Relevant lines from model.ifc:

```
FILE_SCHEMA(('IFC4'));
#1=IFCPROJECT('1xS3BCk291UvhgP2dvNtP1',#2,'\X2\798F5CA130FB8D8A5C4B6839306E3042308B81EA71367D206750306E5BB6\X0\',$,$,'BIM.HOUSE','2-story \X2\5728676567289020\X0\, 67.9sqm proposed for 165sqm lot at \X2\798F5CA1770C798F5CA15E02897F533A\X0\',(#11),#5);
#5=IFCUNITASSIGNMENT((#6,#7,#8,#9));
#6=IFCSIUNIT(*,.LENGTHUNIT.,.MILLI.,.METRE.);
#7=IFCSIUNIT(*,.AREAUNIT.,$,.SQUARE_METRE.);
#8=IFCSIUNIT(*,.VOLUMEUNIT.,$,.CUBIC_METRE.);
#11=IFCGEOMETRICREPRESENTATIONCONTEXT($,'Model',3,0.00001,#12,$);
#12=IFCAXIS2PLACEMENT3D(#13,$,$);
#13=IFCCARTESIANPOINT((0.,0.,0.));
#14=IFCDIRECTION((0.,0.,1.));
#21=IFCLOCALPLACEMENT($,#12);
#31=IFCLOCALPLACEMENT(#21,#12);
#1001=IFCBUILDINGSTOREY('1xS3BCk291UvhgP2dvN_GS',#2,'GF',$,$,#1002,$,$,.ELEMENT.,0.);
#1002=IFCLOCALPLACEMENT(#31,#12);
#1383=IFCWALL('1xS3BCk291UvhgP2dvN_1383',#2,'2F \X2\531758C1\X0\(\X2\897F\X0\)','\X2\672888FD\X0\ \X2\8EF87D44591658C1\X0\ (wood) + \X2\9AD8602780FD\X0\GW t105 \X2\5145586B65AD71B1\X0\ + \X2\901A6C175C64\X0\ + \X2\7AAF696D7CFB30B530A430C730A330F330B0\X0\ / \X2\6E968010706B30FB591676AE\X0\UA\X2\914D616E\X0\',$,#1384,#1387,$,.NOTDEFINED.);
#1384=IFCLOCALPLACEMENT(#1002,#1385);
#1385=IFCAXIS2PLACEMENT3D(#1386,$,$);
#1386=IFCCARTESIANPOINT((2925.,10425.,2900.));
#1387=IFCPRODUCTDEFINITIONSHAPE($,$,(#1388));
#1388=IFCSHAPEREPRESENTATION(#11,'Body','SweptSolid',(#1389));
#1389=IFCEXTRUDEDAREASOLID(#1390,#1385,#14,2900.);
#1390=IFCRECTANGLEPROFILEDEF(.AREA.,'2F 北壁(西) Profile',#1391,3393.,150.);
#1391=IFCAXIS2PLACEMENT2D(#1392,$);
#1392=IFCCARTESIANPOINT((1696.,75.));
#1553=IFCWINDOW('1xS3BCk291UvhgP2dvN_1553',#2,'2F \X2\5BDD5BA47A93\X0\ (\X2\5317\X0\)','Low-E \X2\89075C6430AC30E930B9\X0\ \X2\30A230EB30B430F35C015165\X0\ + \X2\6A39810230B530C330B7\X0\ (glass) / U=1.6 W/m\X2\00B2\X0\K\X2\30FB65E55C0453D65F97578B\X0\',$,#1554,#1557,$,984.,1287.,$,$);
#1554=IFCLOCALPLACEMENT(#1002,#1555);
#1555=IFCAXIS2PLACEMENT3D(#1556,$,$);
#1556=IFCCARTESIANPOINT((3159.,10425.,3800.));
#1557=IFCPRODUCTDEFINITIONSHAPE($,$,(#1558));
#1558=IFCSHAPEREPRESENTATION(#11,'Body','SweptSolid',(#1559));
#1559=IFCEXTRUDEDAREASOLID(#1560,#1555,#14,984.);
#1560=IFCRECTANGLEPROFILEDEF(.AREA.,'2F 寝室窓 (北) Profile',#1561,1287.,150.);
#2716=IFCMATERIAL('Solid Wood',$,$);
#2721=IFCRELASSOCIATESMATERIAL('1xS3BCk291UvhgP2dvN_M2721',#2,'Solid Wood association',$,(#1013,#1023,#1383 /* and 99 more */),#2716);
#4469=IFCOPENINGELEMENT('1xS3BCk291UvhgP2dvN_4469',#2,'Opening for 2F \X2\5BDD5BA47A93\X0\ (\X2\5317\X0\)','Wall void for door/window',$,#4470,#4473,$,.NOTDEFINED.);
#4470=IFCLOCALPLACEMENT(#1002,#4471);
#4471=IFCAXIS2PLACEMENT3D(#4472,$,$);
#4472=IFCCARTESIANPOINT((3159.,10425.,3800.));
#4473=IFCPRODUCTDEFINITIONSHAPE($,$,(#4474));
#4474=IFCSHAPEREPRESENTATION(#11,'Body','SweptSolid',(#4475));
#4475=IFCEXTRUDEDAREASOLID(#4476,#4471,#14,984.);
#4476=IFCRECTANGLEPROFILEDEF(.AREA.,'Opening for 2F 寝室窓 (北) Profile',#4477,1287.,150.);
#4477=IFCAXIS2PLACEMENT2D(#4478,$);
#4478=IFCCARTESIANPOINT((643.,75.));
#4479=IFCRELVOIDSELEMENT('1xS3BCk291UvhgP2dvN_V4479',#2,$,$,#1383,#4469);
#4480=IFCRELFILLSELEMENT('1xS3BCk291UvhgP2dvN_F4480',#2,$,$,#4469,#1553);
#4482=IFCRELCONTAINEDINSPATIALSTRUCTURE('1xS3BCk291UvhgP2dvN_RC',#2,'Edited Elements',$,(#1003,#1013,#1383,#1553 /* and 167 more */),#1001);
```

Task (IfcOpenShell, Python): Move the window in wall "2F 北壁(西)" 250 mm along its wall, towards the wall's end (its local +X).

```python
import ifcopenshell
import ifcopenshell.api.geometry
import ifcopenshell.util.placement

model = ifcopenshell.open("model.ifc")

window = model.by_id(1553)
opening = window.FillsVoids[0].RelatingOpeningElement
wall = opening.VoidsElements[0].RelatingBuildingElement

wall_matrix = ifcopenshell.util.placement.get_local_placement(wall.ObjectPlacement)
shift = wall_matrix[:3, 0] * 250.0
before = ifcopenshell.util.placement.get_local_placement(window.ObjectPlacement)[:3, 3].copy()

# The window is not placed relative to its opening, so move both.
for product in (opening, window):
    matrix = ifcopenshell.util.placement.get_local_placement(product.ObjectPlacement)
    matrix[:3, 3] += shift
    ifcopenshell.api.geometry.edit_object_placement(model, product=product, matrix=matrix, is_si=False)

after = ifcopenshell.util.placement.get_local_placement(window.ObjectPlacement)[:3, 3]
print("window moved by", (after - before).round(3) + 0.0)

model.write("model_updated.ifc")
```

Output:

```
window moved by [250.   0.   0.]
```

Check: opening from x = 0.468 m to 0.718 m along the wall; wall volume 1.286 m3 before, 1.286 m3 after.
